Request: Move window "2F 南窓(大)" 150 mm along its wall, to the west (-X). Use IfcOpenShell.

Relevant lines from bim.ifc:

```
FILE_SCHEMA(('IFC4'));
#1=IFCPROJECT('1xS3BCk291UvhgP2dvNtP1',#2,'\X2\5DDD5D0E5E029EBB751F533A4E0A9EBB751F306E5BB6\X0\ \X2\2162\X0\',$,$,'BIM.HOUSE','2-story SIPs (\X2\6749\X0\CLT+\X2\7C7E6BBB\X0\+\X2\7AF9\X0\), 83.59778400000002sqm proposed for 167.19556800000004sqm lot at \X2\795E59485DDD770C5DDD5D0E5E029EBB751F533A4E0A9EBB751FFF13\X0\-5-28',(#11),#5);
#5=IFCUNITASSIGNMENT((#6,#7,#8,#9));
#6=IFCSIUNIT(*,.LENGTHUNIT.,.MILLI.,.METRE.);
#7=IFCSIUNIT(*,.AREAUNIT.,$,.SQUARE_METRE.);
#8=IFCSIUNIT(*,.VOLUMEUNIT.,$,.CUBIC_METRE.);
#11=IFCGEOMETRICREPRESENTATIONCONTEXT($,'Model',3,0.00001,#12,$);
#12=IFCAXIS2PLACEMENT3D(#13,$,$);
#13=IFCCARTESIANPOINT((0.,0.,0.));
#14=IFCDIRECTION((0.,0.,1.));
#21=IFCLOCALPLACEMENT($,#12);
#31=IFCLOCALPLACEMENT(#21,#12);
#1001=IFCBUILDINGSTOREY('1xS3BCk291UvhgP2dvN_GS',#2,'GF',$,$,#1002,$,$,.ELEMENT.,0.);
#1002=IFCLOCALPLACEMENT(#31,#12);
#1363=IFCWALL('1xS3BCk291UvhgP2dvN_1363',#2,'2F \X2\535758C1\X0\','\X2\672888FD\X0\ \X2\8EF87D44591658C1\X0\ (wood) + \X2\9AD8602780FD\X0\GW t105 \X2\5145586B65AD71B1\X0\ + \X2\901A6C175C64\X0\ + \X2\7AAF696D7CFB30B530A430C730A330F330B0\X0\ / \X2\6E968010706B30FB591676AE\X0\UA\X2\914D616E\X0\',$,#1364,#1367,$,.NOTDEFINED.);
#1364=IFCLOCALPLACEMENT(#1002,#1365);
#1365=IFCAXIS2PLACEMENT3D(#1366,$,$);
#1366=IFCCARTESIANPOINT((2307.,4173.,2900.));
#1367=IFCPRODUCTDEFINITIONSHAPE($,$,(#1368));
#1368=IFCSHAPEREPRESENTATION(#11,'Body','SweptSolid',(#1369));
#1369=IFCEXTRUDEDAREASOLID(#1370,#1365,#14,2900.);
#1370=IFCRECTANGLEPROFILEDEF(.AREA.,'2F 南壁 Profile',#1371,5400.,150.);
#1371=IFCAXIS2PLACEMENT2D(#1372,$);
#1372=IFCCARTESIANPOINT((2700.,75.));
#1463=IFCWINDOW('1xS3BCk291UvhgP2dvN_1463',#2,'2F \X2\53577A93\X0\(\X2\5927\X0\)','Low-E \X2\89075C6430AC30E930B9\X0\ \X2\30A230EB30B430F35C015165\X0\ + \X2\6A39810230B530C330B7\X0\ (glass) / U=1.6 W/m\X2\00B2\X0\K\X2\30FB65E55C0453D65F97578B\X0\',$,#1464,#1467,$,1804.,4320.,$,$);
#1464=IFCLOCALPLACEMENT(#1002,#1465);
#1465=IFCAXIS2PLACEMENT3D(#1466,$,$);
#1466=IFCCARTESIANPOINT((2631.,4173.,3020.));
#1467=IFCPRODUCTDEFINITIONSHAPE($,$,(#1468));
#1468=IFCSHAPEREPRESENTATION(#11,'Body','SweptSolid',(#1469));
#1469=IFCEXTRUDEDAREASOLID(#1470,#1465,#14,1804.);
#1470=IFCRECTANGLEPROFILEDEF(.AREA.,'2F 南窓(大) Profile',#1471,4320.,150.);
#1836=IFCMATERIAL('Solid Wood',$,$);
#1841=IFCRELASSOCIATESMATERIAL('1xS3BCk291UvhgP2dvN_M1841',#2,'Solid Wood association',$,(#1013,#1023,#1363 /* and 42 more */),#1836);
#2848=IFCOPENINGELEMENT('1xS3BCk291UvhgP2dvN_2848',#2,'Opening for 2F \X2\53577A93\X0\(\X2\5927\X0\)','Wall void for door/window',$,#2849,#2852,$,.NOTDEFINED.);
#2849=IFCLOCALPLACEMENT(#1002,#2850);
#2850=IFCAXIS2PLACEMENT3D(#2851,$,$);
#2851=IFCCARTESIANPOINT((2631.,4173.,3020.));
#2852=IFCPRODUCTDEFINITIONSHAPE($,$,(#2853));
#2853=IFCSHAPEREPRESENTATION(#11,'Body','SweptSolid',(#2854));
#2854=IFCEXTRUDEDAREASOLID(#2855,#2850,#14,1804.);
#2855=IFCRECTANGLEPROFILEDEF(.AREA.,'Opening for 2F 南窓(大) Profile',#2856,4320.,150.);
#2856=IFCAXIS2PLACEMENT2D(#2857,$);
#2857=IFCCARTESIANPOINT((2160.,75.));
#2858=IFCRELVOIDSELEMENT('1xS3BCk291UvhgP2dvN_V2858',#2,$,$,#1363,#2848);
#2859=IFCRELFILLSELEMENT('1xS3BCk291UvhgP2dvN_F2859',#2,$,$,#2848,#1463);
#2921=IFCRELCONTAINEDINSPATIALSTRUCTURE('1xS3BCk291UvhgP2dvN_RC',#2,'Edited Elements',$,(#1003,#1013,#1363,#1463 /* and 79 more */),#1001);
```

```python
import ifcopenshell
import ifcopenshell.api.geometry
import ifcopenshell.util.placement
import ifcopenshell.util.unit

model = ifcopenshell.open("bim.ifc")
unit_scale = ifcopenshell.util.unit.calculate_unit_scale(model)

window = model.by_guid("1xS3BCk291UvhgP2dvN_1463")
opening = window.FillsVoids[0].RelatingOpeningElement
wall = opening.VoidsElements[0].RelatingBuildingElement

wall_matrix = ifcopenshell.util.placement.get_local_placement(wall.ObjectPlacement)
shift = wall_matrix[:3, 0] * -0.15 / unit_scale
before = ifcopenshell.util.placement.get_local_placement(window.ObjectPlacement)[:3, 3].copy()

# The window is not placed relative to its opening, so move both.
for product in (opening, window):
    matrix = ifcopenshell.util.placement.get_local_placement(product.ObjectPlacement)
    matrix[:3, 3] += shift
    ifcopenshell.api.geometry.edit_object_placement(model, product=product, matrix=matrix, is_si=False)

after = ifcopenshell.util.placement.get_local_placement(window.ObjectPlacement)[:3, 3]
print("window moved by", (after - before).round(3) + 0.0)

model.write("bim_v2.ifc")
```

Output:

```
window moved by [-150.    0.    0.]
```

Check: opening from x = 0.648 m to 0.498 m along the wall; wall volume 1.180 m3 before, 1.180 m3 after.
